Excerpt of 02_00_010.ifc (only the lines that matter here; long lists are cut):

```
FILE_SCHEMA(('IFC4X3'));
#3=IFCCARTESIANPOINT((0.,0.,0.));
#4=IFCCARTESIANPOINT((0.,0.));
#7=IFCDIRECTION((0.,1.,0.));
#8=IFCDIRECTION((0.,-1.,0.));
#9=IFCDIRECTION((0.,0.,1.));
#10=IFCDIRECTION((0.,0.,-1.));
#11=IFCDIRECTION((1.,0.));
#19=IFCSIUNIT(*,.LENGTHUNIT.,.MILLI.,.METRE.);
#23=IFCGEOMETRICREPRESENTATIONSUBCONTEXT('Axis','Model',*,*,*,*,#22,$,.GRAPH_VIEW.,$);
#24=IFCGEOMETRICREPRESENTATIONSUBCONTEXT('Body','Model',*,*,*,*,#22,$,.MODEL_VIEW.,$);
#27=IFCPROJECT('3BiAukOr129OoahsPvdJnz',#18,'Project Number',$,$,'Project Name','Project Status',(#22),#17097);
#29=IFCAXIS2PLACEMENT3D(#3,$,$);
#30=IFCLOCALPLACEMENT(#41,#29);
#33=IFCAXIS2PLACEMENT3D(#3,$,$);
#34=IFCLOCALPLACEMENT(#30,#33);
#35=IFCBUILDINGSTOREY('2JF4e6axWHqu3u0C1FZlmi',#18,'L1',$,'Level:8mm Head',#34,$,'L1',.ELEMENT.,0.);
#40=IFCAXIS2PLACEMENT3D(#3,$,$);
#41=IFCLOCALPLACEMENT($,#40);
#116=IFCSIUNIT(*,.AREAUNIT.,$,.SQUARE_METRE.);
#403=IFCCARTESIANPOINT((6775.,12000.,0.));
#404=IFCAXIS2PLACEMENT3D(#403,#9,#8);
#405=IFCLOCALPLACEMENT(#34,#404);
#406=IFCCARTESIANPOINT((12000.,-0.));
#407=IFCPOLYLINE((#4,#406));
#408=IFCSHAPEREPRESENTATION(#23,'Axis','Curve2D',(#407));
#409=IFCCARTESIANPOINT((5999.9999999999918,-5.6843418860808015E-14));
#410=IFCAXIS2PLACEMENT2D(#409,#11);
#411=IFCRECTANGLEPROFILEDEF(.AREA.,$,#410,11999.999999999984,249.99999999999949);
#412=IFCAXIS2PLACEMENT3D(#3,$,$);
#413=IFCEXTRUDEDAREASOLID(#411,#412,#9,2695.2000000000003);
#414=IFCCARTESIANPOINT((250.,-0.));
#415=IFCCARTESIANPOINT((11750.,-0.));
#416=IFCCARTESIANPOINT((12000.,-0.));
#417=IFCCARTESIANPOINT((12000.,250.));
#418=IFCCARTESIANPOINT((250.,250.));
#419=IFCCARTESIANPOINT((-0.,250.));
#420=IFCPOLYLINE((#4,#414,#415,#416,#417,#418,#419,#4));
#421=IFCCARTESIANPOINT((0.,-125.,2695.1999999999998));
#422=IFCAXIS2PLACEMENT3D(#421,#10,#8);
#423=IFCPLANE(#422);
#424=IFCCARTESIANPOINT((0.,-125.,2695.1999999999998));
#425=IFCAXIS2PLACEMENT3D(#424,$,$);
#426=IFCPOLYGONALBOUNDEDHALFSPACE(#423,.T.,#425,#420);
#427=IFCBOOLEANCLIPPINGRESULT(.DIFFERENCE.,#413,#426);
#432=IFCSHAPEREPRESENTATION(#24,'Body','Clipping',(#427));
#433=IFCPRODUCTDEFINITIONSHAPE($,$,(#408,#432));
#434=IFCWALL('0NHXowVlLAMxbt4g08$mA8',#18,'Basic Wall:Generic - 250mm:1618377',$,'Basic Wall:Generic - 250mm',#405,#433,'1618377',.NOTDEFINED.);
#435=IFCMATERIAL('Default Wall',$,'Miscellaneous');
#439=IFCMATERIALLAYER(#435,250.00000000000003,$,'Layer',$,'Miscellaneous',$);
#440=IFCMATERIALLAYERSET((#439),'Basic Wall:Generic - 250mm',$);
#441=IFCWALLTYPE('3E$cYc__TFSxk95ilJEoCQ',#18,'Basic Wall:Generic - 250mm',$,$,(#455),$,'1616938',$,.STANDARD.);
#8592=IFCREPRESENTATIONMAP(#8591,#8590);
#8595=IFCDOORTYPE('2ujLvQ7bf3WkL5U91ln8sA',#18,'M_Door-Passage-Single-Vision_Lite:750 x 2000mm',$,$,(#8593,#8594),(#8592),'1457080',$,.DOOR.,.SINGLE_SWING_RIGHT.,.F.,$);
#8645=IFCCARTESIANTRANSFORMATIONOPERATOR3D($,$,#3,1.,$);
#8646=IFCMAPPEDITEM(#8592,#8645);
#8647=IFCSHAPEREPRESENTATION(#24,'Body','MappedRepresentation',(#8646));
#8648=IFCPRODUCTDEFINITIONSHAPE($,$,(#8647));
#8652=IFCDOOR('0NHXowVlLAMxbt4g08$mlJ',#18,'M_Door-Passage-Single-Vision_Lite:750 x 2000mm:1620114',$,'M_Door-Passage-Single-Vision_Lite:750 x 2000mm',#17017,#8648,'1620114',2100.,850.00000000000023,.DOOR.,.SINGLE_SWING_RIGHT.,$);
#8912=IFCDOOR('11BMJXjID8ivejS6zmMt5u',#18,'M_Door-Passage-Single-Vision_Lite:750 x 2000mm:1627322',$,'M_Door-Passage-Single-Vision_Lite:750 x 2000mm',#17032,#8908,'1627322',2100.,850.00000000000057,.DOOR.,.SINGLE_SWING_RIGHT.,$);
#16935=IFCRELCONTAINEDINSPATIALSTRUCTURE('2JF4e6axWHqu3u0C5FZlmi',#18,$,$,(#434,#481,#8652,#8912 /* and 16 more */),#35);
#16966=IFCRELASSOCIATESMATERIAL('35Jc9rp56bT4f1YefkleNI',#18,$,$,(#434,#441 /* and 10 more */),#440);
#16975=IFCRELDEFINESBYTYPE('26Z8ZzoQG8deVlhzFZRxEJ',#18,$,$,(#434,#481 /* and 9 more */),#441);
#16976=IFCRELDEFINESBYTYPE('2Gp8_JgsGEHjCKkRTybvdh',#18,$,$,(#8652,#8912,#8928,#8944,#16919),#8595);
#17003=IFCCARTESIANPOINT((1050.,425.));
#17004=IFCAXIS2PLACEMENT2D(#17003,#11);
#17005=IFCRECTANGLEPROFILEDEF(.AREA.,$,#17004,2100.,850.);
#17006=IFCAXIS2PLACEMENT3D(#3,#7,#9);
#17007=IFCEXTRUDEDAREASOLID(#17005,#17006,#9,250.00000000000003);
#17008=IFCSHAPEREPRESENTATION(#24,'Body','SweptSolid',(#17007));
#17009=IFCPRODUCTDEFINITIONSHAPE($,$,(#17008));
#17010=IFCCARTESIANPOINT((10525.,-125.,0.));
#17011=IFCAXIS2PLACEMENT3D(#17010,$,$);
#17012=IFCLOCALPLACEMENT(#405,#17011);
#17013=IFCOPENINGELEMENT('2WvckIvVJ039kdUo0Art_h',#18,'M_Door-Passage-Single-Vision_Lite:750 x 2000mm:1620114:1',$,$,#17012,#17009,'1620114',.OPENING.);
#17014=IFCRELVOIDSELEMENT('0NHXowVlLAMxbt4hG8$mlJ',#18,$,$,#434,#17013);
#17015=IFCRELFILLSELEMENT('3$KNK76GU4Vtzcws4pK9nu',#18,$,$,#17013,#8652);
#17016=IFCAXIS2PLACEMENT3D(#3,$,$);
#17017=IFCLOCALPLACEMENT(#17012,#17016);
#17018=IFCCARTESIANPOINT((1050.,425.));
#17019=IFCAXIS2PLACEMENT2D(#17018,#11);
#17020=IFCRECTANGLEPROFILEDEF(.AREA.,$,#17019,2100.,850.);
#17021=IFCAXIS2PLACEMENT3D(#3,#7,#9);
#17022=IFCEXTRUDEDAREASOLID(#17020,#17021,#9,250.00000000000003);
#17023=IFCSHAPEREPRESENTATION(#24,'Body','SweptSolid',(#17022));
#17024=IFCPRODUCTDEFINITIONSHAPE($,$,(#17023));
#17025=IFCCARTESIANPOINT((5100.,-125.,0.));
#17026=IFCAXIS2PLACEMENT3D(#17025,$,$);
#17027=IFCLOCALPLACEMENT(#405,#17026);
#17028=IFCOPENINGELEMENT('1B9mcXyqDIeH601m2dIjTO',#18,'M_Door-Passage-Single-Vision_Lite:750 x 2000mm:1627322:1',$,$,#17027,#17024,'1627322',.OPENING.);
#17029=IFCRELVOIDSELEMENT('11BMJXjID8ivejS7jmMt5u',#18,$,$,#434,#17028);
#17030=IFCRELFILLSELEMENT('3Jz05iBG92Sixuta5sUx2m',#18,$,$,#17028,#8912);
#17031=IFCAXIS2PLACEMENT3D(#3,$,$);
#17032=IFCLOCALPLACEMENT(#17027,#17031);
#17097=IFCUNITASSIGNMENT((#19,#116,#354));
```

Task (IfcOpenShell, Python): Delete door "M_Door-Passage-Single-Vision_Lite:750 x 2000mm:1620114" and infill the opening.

```python
import ifcopenshell
import ifcopenshell.api.feature
import ifcopenshell.api.root
import ifcopenshell.geom
import ifcopenshell.util.shape

model = ifcopenshell.open("02_00_010.ifc")
settings = ifcopenshell.geom.settings()


def volume(element):
    """Net volume in cubic metres, openings subtracted."""
    shape = ifcopenshell.geom.create_shape(settings, element)
    return ifcopenshell.util.shape.get_volume(shape.geometry)


door = model.by_guid("0NHXowVlLAMxbt4g08$mlJ")
opening = door.FillsVoids[0].RelatingOpeningElement
wall = opening.VoidsElements[0].RelatingBuildingElement
before = volume(wall)

ifcopenshell.api.root.remove_product(model, product=door)
ifcopenshell.api.feature.remove_feature(model, feature=opening)

after = volume(wall)

print(f"wall volume {before:.3f} -> {after:.3f} m3")

model.write("02_00_010_v2.ifc")
```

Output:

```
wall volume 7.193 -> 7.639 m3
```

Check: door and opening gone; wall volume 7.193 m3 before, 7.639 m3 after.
